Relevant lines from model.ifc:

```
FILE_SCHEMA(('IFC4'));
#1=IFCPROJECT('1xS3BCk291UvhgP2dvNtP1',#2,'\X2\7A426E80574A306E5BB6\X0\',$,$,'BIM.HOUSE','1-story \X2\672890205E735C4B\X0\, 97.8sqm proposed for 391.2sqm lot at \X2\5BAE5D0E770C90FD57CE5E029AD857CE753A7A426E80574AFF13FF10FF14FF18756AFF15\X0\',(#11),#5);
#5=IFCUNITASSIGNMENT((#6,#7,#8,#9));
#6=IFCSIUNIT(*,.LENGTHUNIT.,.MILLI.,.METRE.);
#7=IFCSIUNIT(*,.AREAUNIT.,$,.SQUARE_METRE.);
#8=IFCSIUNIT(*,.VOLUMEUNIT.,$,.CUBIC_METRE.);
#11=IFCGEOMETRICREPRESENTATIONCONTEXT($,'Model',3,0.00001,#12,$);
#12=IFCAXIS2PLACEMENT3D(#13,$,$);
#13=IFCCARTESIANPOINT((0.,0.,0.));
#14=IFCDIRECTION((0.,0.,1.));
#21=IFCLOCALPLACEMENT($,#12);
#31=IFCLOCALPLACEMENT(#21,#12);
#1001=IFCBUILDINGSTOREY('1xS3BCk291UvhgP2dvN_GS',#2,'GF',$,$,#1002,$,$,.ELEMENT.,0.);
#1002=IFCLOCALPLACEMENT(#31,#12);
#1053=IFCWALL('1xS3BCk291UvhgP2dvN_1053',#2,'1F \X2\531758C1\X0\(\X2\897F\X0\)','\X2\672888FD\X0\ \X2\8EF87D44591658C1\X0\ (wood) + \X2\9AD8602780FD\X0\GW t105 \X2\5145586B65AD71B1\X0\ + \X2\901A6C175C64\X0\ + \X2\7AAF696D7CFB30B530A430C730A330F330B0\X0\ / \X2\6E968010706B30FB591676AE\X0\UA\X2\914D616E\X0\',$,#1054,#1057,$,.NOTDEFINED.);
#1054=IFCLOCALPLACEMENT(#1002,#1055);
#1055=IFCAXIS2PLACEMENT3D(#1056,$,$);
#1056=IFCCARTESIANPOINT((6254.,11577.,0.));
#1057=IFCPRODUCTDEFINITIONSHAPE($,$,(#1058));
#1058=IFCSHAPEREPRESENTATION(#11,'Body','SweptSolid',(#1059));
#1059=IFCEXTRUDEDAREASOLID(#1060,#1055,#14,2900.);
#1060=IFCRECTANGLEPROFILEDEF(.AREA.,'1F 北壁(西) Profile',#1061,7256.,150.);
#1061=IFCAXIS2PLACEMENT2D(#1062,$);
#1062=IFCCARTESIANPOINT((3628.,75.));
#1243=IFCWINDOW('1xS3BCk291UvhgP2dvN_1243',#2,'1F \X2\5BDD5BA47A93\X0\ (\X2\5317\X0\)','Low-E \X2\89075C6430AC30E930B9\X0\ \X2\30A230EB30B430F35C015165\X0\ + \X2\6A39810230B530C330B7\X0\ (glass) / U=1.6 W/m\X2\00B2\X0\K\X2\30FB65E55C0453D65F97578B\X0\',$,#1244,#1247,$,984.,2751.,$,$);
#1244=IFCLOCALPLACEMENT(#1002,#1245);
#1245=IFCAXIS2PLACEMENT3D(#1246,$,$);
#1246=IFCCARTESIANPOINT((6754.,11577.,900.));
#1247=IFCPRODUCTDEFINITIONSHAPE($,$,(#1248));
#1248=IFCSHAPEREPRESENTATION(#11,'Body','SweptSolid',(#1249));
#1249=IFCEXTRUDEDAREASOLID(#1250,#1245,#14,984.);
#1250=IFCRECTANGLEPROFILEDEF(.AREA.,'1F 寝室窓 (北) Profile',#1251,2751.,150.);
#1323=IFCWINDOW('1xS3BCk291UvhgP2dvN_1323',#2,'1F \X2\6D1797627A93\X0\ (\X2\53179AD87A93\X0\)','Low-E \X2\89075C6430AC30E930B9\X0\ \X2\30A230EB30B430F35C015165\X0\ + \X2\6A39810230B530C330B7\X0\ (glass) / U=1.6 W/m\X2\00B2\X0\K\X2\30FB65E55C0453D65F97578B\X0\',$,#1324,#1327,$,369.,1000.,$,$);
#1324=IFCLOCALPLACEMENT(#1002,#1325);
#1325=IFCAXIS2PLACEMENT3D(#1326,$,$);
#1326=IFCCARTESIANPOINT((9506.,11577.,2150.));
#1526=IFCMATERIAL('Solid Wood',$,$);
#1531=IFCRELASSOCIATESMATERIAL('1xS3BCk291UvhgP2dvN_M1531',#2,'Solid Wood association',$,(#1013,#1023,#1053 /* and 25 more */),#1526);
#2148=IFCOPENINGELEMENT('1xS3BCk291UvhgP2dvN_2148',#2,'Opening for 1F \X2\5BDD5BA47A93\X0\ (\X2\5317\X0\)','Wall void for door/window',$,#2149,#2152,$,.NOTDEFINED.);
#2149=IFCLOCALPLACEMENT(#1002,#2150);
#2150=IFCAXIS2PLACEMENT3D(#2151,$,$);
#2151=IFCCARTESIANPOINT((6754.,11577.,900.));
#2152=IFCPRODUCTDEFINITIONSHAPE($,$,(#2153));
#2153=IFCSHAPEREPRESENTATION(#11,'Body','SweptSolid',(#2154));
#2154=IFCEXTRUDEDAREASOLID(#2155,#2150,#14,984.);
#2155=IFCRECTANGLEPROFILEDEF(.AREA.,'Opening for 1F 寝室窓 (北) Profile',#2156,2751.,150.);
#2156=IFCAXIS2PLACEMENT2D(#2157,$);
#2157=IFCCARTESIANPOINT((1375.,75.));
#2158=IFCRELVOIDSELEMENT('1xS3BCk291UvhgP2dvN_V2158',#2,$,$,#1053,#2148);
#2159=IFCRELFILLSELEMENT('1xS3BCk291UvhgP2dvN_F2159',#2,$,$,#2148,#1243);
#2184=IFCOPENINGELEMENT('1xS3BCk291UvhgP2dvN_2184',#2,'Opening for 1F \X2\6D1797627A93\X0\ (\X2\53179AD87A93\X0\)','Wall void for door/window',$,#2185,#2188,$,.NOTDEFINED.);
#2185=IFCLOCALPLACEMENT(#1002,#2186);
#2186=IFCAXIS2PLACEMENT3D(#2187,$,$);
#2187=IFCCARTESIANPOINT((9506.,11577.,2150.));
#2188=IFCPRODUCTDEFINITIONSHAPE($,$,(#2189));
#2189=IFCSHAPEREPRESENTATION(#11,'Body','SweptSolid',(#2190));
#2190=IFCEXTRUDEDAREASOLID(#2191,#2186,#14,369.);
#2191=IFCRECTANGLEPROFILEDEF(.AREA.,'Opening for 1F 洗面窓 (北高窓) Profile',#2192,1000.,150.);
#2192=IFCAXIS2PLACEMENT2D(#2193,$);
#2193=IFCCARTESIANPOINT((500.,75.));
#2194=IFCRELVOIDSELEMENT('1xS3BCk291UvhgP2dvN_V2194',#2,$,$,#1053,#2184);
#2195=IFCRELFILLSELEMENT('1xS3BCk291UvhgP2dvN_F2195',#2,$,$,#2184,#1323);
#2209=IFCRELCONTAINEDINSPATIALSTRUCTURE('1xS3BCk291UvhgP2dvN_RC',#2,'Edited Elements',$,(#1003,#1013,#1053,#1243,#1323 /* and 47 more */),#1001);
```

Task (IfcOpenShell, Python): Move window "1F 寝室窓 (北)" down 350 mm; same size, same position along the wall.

```python
import numpy as np
import ifcopenshell
import ifcopenshell.api.geometry
import ifcopenshell.util.placement
import ifcopenshell.util.unit

model = ifcopenshell.open("model.ifc")
unit_scale = ifcopenshell.util.unit.calculate_unit_scale(model)

window = model.by_guid("1xS3BCk291UvhgP2dvN_1243")
opening = window.FillsVoids[0].RelatingOpeningElement
dz = -0.35 / unit_scale

shift = np.array([0.0, 0.0, dz])
# The window is not placed relative to its opening, so move both.
for product in (opening, window):
    matrix = ifcopenshell.util.placement.get_local_placement(product.ObjectPlacement)
    matrix[:3, 3] += shift
    ifcopenshell.api.geometry.edit_object_placement(model, product=product, matrix=matrix, is_si=False)

print(f"moved by {dz * unit_scale:+.3f} m")

model.write("model_v2.ifc")
```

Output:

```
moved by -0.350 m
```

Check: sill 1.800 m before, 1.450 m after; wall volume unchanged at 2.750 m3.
